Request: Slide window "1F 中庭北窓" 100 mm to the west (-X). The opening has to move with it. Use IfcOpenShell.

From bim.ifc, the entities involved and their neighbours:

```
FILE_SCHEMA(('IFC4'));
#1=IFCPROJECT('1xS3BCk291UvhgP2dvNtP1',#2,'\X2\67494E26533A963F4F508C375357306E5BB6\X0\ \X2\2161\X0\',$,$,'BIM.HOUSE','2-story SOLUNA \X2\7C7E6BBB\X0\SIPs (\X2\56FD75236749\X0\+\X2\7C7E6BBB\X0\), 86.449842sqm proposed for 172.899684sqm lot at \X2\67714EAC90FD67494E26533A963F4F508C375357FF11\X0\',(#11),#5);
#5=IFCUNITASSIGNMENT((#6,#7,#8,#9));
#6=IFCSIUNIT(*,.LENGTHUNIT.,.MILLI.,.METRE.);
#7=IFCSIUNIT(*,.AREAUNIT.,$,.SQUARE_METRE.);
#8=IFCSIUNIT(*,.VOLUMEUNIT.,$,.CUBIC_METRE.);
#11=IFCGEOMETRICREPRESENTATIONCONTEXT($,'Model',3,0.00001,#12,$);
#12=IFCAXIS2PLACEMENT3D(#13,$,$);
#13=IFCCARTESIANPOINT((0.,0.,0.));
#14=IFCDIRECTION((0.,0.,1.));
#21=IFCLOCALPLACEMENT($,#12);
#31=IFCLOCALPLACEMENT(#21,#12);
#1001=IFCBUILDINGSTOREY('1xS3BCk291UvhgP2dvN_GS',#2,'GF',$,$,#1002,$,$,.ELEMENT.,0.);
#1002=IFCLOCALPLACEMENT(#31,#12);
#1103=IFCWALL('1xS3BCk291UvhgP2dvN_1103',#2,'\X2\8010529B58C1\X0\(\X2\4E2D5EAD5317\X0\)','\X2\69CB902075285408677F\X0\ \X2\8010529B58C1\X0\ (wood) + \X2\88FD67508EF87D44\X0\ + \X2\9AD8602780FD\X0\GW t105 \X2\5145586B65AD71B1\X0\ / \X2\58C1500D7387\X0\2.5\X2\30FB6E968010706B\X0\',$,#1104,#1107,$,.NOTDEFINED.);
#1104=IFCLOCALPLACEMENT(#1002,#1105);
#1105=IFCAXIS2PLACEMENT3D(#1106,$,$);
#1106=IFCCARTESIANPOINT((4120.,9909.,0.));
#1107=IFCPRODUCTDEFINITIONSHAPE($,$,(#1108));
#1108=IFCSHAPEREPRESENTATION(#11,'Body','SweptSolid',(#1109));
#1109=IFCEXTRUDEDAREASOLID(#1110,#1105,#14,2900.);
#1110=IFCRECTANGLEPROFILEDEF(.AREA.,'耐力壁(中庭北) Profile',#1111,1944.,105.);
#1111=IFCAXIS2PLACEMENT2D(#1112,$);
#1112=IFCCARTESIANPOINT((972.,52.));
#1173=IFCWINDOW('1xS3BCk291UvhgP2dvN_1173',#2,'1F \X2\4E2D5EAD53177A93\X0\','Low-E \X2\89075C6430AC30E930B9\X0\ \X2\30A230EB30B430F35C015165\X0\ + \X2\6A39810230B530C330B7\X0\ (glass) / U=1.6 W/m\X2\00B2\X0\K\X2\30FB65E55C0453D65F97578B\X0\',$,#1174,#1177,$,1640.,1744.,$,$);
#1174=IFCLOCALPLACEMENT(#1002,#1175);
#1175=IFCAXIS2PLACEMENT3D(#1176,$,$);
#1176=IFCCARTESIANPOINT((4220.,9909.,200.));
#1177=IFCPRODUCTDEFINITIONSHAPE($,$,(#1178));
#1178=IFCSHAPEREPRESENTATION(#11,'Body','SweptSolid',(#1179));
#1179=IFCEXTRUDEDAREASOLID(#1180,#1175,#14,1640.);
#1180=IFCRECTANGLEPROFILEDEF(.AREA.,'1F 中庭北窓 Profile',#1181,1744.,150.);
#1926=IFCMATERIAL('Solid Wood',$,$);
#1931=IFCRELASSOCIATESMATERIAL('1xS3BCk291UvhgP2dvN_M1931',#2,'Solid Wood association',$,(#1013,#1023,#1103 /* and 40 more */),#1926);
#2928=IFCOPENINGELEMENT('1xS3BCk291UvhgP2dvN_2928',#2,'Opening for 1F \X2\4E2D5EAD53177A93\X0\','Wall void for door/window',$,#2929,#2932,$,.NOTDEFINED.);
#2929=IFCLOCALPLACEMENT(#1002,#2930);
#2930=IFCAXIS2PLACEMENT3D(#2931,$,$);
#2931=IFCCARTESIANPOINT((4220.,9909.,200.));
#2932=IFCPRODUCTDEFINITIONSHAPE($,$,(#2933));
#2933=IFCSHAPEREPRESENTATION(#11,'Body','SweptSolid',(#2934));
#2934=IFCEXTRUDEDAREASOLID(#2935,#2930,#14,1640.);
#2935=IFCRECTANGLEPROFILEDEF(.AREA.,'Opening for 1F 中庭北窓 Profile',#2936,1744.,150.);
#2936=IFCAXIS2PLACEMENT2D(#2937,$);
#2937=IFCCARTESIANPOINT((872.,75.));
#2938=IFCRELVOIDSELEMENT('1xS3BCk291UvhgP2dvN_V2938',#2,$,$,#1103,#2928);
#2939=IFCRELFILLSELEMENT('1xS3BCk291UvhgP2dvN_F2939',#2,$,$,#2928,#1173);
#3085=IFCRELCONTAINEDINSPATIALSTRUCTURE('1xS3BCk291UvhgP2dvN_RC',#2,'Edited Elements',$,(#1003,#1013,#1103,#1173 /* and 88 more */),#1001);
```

```python
import ifcopenshell
import ifcopenshell.api.geometry
import ifcopenshell.util.placement

model = ifcopenshell.open("bim.ifc")

window = model.by_guid("1xS3BCk291UvhgP2dvN_1173")
opening = window.FillsVoids[0].RelatingOpeningElement
wall = opening.VoidsElements[0].RelatingBuildingElement

wall_matrix = ifcopenshell.util.placement.get_local_placement(wall.ObjectPlacement)
shift = wall_matrix[:3, 0] * -100.0
before = ifcopenshell.util.placement.get_local_placement(window.ObjectPlacement)[:3, 3].copy()

# The window is not placed relative to its opening, so move both.
for product in (opening, window):
    matrix = ifcopenshell.util.placement.get_local_placement(product.ObjectPlacement)
    matrix[:3, 3] += shift
    ifcopenshell.api.geometry.edit_object_placement(model, product=product, matrix=matrix, is_si=False)

after = ifcopenshell.util.placement.get_local_placement(window.ObjectPlacement)[:3, 3]
print("window moved by", (after - before).round(3) + 0.0)

model.write("bim_v2.ifc")
```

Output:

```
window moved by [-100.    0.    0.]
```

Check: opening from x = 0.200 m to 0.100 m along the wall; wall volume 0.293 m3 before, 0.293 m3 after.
